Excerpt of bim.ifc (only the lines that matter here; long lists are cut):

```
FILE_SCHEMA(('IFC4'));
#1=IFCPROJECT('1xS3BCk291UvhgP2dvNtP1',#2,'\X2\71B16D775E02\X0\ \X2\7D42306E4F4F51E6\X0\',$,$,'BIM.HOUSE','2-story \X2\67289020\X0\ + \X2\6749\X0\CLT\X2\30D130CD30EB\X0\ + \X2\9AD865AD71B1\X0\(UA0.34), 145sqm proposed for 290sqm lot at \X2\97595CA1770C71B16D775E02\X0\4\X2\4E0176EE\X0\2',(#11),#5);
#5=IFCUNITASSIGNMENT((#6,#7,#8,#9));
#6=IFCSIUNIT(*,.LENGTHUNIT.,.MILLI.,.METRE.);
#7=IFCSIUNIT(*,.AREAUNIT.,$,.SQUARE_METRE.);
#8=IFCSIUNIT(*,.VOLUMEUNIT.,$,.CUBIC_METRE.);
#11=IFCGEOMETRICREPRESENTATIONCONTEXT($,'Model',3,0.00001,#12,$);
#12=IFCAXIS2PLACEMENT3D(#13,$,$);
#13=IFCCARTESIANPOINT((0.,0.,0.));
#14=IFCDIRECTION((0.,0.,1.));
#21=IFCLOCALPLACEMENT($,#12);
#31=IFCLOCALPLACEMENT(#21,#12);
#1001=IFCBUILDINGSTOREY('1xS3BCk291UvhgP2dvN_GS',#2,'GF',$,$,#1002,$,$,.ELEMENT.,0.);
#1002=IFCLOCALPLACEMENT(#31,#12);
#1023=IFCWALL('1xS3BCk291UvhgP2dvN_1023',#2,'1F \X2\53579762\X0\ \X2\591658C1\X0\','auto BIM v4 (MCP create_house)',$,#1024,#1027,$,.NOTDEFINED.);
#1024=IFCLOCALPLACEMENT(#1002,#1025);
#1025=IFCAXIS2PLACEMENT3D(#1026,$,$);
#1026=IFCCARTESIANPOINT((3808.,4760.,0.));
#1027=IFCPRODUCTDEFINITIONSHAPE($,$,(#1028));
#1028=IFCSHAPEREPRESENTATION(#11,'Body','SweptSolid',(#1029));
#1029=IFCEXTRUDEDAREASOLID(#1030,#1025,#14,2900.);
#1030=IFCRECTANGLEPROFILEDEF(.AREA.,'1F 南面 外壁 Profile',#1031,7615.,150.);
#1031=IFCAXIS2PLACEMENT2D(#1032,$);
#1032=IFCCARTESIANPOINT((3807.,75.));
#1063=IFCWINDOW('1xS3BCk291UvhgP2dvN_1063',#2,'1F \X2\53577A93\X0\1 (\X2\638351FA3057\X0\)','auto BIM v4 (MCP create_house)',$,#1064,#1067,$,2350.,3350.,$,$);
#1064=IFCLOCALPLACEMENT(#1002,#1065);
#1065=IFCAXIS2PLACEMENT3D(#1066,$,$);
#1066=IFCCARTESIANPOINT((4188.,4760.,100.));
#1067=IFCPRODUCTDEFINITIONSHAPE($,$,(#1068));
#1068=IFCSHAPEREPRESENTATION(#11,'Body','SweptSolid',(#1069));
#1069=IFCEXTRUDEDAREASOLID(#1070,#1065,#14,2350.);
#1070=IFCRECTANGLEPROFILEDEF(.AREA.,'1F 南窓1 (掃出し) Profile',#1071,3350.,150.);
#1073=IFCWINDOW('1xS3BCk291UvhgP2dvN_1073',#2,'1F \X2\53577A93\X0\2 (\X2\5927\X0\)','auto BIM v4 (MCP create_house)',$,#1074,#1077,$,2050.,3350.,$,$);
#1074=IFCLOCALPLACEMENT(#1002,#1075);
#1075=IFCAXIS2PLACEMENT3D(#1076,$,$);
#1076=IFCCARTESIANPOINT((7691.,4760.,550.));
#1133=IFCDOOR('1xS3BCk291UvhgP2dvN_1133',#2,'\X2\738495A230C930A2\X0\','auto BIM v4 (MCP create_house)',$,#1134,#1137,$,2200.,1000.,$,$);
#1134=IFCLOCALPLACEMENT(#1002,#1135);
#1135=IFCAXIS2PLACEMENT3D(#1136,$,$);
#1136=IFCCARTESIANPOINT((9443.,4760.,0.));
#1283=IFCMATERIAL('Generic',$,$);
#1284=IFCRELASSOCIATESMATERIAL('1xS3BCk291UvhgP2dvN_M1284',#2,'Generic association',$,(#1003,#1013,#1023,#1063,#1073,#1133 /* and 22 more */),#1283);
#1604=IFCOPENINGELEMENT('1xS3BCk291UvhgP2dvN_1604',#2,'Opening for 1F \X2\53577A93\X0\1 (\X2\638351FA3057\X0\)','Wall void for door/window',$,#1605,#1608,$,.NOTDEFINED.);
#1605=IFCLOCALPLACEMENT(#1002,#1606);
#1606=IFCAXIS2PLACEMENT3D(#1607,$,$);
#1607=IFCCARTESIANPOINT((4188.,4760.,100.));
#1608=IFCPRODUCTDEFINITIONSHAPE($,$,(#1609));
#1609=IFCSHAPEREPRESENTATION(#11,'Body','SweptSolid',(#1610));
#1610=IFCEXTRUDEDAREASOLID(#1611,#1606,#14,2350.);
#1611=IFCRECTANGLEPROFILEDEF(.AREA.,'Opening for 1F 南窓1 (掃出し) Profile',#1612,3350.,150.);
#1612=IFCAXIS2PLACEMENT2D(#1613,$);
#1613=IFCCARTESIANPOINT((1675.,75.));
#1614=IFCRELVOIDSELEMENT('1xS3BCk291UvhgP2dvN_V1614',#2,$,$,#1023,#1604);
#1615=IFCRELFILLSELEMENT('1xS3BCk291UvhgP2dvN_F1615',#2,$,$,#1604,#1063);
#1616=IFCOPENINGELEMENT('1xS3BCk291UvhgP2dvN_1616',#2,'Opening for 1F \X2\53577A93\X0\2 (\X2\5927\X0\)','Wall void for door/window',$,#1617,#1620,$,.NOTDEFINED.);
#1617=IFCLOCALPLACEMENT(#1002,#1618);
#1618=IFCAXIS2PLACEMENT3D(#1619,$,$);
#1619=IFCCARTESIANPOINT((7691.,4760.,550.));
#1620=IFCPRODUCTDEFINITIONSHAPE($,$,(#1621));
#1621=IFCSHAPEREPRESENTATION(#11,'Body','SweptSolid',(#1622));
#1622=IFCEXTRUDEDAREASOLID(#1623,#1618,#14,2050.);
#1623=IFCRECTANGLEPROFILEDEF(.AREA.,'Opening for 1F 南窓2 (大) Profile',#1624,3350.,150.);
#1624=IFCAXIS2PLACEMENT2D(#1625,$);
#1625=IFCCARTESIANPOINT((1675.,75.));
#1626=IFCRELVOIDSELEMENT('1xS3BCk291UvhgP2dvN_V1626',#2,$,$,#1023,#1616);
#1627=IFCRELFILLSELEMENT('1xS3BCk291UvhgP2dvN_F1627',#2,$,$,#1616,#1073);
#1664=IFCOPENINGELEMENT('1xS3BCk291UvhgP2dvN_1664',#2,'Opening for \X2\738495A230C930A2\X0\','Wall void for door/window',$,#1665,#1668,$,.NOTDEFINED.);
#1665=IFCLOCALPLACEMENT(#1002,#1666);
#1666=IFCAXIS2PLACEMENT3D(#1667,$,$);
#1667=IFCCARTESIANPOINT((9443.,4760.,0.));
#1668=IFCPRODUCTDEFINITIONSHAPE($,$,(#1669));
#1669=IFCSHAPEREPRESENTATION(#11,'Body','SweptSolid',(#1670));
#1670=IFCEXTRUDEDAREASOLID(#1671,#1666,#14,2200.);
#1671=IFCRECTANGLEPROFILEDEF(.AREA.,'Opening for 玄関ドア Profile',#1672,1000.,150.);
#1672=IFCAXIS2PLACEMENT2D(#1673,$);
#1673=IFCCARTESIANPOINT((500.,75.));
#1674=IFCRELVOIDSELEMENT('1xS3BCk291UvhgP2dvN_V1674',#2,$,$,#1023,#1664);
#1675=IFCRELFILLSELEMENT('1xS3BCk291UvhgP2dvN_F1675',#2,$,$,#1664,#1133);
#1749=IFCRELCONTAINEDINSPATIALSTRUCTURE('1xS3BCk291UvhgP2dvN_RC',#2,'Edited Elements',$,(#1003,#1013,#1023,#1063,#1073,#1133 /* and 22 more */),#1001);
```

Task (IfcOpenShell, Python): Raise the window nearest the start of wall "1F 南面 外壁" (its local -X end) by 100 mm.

```python
import numpy as np
import ifcopenshell
import ifcopenshell.api.geometry
import ifcopenshell.util.placement
import ifcopenshell.util.unit

model = ifcopenshell.open("bim.ifc")
unit_scale = ifcopenshell.util.unit.calculate_unit_scale(model)

window = model.by_id(1063)
opening = window.FillsVoids[0].RelatingOpeningElement
dz = 100.0

shift = np.array([0.0, 0.0, dz])
# The window is not placed relative to its opening, so move both.
for product in (opening, window):
    matrix = ifcopenshell.util.placement.get_local_placement(product.ObjectPlacement)
    matrix[:3, 3] += shift
    ifcopenshell.api.geometry.edit_object_placement(model, product=product, matrix=matrix, is_si=False)

print(f"moved by {dz * unit_scale:+.3f} m")

model.write("bim-out.ifc")
```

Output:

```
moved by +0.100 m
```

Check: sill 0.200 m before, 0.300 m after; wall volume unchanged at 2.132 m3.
